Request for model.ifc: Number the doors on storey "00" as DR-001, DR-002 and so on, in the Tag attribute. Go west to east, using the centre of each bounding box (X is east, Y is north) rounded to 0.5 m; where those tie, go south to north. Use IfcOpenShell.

First a look at what the model holds.

```python
import ifcopenshell
import ifcopenshell.util.element
import ifcopenshell.util.placement

model = ifcopenshell.open("model.ifc")
print(model.schema)
storey = next(s for s in model.by_type("IfcBuildingStorey") if s.Name == "00")
doors = [e for e in ifcopenshell.util.element.get_decomposition(storey) if e.is_a("IfcDoor")]
for e in sorted(doors, key=lambda e: e.id()):
    origin = ifcopenshell.util.placement.get_local_placement(e.ObjectPlacement)[:3, 3]
    print(e.id(), e.Tag, e.Name, origin.round(2) + 0.0, sep=" | ")
```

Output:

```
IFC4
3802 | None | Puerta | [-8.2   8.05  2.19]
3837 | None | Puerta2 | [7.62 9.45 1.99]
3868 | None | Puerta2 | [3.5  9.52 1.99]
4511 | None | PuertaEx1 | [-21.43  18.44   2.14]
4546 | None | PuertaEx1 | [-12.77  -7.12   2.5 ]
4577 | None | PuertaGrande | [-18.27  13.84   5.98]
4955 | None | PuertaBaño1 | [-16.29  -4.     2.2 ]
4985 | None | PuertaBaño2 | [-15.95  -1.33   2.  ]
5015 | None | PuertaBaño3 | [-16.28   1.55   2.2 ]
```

```python
import ifcopenshell
import ifcopenshell.geom
import ifcopenshell.util.element
import ifcopenshell.util.shape

model = ifcopenshell.open("model.ifc")
settings = ifcopenshell.geom.settings()
settings.set("use-world-coords", True)


def centre(element):
    shape = ifcopenshell.geom.create_shape(settings, element)
    return ifcopenshell.util.shape.get_bbox_centroid(shape.geometry)


storey = next(s for s in model.by_type("IfcBuildingStorey") if s.Name == "00")
doors = [e for e in ifcopenshell.util.element.get_decomposition(storey) if e.is_a("IfcDoor")]

# Insertion points can sit at a corner or the storey origin, so sort by the geometry (in metres).
centres = {e: centre(e) for e in doors}
doors.sort(key=lambda e: (round(centres[e][0] / 0.5), centres[e][1]))

for i, e in enumerate(doors, start=1):
    number = f"DR-0{i:02d}"
    e.Tag = number
    print(e.id(), number)

model.write("model-out.ifc")
```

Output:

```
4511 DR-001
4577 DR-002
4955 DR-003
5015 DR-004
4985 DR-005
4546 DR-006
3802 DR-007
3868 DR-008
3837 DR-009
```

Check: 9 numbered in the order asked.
